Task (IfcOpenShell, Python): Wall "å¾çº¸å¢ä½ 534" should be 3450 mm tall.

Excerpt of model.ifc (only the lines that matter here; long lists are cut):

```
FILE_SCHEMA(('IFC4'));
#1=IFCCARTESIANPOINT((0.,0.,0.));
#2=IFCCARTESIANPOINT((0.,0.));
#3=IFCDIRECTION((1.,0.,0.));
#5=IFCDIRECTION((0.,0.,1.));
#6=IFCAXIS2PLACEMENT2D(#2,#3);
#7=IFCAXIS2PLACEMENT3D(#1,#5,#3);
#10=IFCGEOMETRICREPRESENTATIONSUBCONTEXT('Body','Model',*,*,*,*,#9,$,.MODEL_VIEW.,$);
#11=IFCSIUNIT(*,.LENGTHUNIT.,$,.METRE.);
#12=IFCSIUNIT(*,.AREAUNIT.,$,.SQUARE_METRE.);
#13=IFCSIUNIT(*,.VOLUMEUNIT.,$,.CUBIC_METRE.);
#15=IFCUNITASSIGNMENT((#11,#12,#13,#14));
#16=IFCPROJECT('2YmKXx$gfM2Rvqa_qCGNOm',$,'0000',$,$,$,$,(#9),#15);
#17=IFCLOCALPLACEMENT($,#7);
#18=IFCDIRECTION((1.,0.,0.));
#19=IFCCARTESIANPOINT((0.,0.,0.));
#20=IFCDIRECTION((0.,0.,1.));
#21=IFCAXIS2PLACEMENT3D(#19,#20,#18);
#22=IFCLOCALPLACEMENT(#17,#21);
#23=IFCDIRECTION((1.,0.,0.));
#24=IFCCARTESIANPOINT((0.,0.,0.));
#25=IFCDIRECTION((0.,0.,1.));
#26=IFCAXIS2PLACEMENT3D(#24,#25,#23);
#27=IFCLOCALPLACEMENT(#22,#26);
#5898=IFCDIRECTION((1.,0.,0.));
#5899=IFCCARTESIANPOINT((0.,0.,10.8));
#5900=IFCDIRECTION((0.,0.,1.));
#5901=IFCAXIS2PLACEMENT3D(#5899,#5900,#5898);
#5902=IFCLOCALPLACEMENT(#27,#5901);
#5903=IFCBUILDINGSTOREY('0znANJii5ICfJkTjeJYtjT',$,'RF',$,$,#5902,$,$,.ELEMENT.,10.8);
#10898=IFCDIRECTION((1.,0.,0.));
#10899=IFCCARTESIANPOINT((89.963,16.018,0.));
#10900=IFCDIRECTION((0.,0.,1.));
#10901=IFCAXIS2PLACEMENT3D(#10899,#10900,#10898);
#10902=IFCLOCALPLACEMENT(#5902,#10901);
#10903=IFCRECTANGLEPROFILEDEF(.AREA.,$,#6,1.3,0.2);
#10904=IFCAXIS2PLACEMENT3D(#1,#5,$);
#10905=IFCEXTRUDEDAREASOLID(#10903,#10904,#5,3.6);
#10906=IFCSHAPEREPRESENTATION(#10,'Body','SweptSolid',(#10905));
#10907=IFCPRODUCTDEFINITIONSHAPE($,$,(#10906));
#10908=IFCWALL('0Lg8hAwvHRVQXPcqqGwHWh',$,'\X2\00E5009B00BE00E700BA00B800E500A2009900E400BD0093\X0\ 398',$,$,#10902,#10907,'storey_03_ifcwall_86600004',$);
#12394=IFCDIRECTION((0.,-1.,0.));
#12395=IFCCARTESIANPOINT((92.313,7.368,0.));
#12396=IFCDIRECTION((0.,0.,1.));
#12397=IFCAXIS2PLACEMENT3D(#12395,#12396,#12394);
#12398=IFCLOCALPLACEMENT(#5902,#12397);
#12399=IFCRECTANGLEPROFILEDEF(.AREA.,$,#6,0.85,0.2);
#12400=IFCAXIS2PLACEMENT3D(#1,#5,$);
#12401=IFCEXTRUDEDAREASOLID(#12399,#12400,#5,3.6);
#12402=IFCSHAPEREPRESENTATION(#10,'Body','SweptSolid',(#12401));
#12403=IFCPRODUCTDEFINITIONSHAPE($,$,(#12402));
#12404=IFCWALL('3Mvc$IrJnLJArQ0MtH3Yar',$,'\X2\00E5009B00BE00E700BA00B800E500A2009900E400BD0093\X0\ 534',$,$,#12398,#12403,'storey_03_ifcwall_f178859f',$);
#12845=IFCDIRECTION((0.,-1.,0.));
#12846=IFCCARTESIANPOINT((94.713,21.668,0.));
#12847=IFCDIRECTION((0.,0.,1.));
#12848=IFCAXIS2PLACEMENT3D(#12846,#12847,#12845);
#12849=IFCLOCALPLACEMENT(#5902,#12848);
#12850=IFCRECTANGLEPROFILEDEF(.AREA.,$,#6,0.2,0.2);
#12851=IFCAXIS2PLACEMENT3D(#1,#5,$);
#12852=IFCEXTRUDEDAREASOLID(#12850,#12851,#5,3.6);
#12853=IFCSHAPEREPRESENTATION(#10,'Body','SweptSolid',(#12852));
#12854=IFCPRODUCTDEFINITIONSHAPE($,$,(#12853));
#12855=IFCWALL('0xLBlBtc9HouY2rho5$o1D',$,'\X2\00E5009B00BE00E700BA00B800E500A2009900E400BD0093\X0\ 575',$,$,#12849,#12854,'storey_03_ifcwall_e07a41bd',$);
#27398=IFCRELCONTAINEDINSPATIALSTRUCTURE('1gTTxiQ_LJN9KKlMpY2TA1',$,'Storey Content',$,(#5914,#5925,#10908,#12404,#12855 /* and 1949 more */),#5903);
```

```python
import ifcopenshell
import ifcopenshell.geom
import ifcopenshell.util.representation
import ifcopenshell.util.shape
import ifcopenshell.util.unit

model = ifcopenshell.open("model.ifc")
unit_scale = ifcopenshell.util.unit.calculate_unit_scale(model)
settings = ifcopenshell.geom.settings()


def volume(element):
    """Net volume in cubic metres, openings subtracted."""
    shape = ifcopenshell.geom.create_shape(settings, element)
    return ifcopenshell.util.shape.get_volume(shape.geometry)


wall = model.by_id(12404)
before = volume(wall)

body = ifcopenshell.util.representation.get_representation(wall, "Model", "Body")
solid = body.Items[0]
old_height = solid.Depth
solid.Depth = 3.45 / unit_scale
after = volume(wall)

print(f"height {old_height:g} -> {solid.Depth:g}, volume {before:.3f} -> {after:.3f} m3")

model.write("model_edited.ifc")
```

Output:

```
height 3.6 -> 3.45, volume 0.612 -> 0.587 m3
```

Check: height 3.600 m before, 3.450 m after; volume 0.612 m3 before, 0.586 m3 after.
